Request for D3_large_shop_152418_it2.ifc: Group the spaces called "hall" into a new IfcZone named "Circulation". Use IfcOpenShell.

First a look at what the model holds.

```python
import ifcopenshell

model = ifcopenshell.open("D3_large_shop_152418_it2.ifc")
print(model.schema)
seen = {}
for space in model.by_type("IfcSpace"):
    seen[space.LongName] = seen.get(space.LongName, 0) + 1
for name, count in sorted(seen.items(), key=str):
    print(count, "x", name)
print("zones:", [z.Name for z in model.by_type("IfcZone")][:20])
```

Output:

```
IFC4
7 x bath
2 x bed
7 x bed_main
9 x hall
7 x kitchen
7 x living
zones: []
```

```python
import ifcopenshell
import ifcopenshell.api.group
import ifcopenshell.api.root

model = ifcopenshell.open("D3_large_shop_152418_it2.ifc")

names = {"hall"}
spaces = [s for s in model.by_type("IfcSpace") if s.LongName in names]

zone = ifcopenshell.api.root.create_entity(model, ifc_class="IfcZone", name="Circulation")
ifcopenshell.api.group.assign_group(model, products=spaces, group=zone)
print(len(spaces), "spaces in", zone.Name)

model.write("D3_large_shop_152418_it2-out.ifc")
```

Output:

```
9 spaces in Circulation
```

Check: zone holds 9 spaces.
